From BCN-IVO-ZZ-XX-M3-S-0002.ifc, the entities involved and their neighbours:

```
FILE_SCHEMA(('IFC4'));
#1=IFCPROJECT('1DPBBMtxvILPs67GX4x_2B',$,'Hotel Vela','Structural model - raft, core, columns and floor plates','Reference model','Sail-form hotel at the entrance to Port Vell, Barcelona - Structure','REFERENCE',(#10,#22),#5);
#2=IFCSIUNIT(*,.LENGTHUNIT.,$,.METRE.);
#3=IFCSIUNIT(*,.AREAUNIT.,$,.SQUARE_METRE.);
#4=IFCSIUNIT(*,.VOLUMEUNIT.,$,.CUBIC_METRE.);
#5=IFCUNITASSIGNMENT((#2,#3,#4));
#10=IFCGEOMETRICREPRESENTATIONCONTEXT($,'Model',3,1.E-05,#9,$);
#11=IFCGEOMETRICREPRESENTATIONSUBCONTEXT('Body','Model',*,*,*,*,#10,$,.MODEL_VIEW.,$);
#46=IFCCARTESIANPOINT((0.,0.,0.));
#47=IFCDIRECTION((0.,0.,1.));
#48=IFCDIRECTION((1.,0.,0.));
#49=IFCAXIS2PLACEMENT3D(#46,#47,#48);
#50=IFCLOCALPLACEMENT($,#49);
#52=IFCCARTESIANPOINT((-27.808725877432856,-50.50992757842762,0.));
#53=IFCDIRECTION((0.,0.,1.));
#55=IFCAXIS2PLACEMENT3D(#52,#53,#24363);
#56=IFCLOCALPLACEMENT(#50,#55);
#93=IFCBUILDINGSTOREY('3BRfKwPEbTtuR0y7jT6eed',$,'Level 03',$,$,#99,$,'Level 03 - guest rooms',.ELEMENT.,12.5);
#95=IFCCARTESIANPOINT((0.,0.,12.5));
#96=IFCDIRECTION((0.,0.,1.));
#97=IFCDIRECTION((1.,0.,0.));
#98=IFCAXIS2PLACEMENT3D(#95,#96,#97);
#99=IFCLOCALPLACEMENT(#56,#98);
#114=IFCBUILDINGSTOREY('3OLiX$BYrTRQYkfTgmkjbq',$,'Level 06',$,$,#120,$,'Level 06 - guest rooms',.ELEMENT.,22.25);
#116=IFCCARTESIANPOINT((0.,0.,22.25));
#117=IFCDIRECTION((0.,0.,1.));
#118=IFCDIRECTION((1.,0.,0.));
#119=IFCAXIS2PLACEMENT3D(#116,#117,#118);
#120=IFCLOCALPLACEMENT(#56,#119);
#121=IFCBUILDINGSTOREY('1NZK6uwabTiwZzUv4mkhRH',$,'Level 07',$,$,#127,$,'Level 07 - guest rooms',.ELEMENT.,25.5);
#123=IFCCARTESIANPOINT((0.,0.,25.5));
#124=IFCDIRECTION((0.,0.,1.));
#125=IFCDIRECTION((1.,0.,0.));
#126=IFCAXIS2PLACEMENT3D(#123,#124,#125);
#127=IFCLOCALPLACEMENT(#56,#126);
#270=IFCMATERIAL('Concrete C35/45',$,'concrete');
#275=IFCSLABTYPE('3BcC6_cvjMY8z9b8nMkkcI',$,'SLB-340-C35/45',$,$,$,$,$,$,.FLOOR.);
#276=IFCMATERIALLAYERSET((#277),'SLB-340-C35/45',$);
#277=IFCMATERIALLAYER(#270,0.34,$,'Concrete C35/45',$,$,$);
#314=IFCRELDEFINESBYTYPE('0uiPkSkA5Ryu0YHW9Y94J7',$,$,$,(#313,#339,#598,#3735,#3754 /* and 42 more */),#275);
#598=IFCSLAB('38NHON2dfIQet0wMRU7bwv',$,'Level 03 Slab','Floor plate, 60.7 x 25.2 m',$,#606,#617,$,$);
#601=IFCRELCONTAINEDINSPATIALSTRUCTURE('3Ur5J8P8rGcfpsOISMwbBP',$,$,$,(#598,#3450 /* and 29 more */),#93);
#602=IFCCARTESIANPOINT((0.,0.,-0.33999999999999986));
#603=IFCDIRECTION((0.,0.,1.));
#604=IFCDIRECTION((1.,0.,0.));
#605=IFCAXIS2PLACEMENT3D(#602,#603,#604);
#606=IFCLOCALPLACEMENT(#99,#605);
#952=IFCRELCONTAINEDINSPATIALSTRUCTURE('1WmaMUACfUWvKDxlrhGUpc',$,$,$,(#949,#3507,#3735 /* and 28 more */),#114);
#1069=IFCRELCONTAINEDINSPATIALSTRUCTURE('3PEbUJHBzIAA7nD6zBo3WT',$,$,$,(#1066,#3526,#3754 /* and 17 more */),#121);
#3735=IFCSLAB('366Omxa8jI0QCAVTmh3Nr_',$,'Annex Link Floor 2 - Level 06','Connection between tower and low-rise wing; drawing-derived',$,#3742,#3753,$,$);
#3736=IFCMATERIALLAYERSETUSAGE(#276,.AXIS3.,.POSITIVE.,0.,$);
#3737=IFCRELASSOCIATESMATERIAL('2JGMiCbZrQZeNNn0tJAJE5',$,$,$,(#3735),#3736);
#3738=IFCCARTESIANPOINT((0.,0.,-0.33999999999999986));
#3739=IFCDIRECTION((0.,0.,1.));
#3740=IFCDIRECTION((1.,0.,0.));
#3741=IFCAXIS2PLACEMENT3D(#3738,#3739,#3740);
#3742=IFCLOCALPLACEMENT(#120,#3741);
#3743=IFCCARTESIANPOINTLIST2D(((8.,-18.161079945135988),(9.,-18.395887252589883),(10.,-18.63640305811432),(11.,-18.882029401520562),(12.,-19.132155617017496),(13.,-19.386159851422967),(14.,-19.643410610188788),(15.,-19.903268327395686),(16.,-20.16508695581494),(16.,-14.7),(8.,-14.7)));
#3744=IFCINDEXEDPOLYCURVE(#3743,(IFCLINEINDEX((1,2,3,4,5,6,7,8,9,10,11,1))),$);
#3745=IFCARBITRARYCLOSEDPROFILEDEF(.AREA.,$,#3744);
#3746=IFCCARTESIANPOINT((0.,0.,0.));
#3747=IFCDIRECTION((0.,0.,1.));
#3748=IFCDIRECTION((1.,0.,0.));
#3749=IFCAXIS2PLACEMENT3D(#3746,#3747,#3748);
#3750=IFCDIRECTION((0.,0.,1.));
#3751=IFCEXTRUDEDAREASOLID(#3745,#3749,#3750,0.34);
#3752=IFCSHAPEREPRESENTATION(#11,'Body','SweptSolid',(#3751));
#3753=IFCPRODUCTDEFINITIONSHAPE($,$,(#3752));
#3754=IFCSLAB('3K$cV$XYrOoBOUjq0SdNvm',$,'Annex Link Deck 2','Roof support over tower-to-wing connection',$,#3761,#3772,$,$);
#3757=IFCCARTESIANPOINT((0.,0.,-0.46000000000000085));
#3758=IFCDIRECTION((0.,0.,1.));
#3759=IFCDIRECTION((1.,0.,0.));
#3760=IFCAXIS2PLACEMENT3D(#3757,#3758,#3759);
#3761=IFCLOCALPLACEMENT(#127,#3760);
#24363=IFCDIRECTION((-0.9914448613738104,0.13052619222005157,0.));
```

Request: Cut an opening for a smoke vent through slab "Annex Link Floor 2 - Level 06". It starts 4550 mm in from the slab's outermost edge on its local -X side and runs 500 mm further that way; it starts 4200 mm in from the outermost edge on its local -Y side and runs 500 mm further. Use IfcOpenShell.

```python
import numpy as np
import ifcopenshell
import ifcopenshell.api.feature
import ifcopenshell.api.geometry
import ifcopenshell.api.root
import ifcopenshell.geom
import ifcopenshell.util.placement
import ifcopenshell.util.representation
import ifcopenshell.util.shape
import ifcopenshell.util.unit

model = ifcopenshell.open("BCN-IVO-ZZ-XX-M3-S-0002.ifc")
unit_scale = ifcopenshell.util.unit.calculate_unit_scale(model)
settings = ifcopenshell.geom.settings()


def volume(element):
    """Net volume in cubic metres, openings subtracted."""
    shape = ifcopenshell.geom.create_shape(settings, element)
    return ifcopenshell.util.shape.get_volume(shape.geometry)


slab = model.by_guid("366Omxa8jI0QCAVTmh3Nr_")
before = volume(slab)

# Extent in the slab's own axes, in metres. The edges named are its -X and -Y sides.
slab_shape = ifcopenshell.geom.create_shape(settings, slab)
vertices = ifcopenshell.util.shape.get_vertices(slab_shape.geometry)
x_min, y_min, bottom = vertices.min(axis=0)
top = vertices[:, 2].max()

opening = ifcopenshell.api.root.create_entity(model, ifc_class="IfcOpeningElement", name="Smoke vent opening", predefined_type="OPENING")
context = ifcopenshell.util.representation.get_context(model, "Model", "Body", "MODEL_VIEW")
width, depth = 0.5, 0.5
outline = [(0.0, 0.0), (width, 0.0), (width, depth), (0.0, depth), (0.0, 0.0)]
# Overshoot both faces by 50 mm so the cut is clean.
shape = ifcopenshell.api.geometry.add_slab_representation(
    model, context=context, depth=top - bottom + 0.1, polyline=outline
)
ifcopenshell.api.geometry.assign_representation(model, product=opening, representation=shape)

matrix = ifcopenshell.util.placement.get_local_placement(slab.ObjectPlacement)
matrix[:, 3] = matrix @ np.append(np.array([x_min + 4.55, y_min + 4.2, bottom - 0.05]) / unit_scale, 1.0)
ifcopenshell.api.geometry.edit_object_placement(model, product=opening, matrix=matrix, is_si=False)
ifcopenshell.api.feature.add_feature(model, feature=opening, element=slab)

after = volume(slab)

print(f"slab volume {before:.3f} -> {after:.3f} m3")

model.write("BCN-IVO-ZZ-XX-M3-S-0002_updated.ifc")
```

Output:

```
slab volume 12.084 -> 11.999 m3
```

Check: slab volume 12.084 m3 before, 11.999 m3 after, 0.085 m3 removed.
